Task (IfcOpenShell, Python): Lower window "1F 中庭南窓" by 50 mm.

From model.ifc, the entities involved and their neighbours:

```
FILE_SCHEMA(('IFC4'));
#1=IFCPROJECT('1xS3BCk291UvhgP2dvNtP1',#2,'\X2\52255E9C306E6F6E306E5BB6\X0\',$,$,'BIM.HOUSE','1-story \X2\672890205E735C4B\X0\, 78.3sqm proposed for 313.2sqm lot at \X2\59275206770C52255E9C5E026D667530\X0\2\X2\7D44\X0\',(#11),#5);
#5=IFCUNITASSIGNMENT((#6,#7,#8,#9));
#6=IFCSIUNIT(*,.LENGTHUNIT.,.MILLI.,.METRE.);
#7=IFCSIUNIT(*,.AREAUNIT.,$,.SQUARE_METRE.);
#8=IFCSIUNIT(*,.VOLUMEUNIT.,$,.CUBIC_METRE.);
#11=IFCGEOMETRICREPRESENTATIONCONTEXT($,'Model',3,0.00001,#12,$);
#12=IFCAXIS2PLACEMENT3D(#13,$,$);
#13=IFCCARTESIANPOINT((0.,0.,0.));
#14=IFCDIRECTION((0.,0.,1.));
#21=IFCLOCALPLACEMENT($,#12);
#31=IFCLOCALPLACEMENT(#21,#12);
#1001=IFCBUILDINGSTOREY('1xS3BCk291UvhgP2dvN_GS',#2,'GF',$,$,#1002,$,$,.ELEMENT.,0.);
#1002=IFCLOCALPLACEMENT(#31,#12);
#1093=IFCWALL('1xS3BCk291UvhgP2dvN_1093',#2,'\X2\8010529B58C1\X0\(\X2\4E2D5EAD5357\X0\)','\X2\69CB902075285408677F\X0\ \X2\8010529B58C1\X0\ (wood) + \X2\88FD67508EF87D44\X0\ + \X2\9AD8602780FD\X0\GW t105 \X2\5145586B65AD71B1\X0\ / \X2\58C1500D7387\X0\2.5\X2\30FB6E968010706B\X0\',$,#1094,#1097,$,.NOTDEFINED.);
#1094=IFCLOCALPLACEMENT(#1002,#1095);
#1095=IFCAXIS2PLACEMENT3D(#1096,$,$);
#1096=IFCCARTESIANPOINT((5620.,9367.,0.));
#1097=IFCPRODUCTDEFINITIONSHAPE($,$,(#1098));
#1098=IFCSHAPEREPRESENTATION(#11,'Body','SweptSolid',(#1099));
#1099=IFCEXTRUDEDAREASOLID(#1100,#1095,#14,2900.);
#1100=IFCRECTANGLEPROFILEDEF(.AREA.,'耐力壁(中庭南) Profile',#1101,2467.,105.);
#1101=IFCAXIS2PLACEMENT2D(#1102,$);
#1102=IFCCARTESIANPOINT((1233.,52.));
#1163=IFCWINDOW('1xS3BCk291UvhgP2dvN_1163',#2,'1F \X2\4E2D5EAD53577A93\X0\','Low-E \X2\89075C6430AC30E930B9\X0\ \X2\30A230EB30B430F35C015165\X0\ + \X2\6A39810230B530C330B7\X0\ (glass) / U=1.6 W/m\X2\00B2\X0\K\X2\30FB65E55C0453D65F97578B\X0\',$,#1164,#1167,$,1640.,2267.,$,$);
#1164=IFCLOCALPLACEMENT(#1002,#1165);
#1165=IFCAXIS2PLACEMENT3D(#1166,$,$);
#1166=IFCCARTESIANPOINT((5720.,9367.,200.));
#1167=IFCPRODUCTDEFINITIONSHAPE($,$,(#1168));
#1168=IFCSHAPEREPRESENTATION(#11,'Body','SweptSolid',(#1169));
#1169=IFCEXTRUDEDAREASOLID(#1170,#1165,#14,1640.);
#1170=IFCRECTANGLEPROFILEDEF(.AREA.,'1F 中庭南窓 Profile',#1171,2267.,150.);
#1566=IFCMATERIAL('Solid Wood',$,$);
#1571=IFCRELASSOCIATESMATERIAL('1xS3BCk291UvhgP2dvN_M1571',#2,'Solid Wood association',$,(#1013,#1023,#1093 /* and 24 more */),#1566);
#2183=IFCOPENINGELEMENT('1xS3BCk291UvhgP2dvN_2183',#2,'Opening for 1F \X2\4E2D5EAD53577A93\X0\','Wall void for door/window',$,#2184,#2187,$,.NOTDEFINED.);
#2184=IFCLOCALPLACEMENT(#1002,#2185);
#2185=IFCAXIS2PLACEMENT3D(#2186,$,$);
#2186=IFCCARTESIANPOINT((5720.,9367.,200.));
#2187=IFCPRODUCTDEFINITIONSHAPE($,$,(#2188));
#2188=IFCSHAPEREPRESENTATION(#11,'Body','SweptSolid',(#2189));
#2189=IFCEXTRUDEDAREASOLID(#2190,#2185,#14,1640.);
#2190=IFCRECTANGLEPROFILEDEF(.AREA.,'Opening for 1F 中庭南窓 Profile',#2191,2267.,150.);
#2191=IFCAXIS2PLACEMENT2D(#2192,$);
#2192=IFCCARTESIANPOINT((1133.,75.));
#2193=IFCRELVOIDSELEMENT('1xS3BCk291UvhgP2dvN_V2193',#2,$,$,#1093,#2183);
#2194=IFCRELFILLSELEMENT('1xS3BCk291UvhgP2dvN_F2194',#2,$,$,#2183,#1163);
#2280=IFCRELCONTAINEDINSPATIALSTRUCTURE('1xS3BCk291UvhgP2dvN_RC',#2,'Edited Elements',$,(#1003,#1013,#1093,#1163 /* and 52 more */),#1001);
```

```python
import numpy as np
import ifcopenshell
import ifcopenshell.api.geometry
import ifcopenshell.util.placement
import ifcopenshell.util.unit

model = ifcopenshell.open("model.ifc")
unit_scale = ifcopenshell.util.unit.calculate_unit_scale(model)

window = model.by_id(1163)
opening = window.FillsVoids[0].RelatingOpeningElement
dz = -50.0

shift = np.array([0.0, 0.0, dz])
# The window is not placed relative to its opening, so move both.
for product in (opening, window):
    matrix = ifcopenshell.util.placement.get_local_placement(product.ObjectPlacement)
    matrix[:3, 3] += shift
    ifcopenshell.api.geometry.edit_object_placement(model, product=product, matrix=matrix, is_si=False)

print(f"moved by {dz * unit_scale:+.3f} m")

model.write("model_v2.ifc")
```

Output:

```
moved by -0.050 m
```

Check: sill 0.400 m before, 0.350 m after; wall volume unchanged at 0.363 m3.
